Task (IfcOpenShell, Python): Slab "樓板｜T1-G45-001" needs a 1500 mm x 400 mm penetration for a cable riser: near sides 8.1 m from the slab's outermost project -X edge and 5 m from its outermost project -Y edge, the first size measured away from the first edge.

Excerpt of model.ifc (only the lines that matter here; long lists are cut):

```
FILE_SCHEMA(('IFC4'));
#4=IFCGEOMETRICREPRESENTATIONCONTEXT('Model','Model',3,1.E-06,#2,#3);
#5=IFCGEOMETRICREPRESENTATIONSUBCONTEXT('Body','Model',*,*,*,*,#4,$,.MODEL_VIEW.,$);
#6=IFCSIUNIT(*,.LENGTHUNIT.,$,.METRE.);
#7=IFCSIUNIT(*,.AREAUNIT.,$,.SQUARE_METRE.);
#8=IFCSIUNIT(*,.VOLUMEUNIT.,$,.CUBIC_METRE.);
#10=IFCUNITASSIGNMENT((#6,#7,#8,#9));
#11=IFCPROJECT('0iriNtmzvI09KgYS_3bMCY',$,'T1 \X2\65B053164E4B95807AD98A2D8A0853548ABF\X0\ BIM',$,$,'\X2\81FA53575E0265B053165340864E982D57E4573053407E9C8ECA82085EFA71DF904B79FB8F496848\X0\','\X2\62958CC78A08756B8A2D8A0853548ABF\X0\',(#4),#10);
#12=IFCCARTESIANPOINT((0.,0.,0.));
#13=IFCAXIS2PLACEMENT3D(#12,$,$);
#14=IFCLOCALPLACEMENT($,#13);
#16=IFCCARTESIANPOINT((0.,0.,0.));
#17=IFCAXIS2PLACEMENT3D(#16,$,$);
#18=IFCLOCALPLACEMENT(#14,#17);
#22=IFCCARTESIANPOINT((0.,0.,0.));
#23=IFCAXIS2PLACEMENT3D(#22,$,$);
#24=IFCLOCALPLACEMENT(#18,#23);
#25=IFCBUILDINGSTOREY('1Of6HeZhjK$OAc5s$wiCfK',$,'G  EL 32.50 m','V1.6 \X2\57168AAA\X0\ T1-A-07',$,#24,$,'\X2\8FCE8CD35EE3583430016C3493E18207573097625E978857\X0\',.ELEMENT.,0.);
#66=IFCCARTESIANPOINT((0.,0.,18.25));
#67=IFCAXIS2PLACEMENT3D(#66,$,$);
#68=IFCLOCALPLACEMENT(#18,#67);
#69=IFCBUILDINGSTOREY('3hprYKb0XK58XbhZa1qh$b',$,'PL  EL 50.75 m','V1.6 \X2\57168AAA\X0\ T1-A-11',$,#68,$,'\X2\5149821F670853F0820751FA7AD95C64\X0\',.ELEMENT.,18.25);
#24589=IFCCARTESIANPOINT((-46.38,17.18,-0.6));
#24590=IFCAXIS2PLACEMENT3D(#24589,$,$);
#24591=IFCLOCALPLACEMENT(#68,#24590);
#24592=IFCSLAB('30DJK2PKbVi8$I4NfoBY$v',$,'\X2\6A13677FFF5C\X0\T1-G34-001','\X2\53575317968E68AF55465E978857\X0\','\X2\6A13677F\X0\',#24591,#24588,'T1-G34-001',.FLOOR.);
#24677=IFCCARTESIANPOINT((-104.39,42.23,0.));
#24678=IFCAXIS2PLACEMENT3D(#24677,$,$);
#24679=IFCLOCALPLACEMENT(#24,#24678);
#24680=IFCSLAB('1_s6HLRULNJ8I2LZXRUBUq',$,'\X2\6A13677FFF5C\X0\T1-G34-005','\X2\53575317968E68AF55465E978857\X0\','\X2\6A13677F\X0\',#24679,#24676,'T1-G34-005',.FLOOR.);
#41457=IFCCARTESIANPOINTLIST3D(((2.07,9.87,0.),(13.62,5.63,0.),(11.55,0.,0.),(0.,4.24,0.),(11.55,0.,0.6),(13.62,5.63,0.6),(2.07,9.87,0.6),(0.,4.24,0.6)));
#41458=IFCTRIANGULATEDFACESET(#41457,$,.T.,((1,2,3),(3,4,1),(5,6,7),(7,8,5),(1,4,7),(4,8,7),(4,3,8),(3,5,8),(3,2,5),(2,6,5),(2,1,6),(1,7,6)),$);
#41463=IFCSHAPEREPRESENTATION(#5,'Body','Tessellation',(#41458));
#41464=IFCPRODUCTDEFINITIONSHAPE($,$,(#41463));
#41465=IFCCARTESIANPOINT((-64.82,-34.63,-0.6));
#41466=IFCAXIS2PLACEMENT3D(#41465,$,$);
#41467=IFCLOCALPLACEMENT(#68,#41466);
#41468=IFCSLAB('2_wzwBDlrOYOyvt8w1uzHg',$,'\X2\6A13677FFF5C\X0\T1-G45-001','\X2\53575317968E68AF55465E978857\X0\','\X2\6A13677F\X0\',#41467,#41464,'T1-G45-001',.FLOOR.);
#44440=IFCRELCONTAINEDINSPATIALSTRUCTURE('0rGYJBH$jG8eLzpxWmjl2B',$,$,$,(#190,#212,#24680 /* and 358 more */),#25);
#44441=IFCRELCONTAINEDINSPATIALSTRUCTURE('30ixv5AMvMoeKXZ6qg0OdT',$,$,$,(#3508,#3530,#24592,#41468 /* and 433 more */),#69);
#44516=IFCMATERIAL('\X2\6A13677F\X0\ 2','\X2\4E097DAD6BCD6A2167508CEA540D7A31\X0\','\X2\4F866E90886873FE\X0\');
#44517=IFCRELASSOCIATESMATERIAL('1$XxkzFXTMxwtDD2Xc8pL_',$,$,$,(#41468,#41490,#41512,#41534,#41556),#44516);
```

```python
import numpy as np
import ifcopenshell
import ifcopenshell.api.feature
import ifcopenshell.api.geometry
import ifcopenshell.api.root
import ifcopenshell.geom
import ifcopenshell.util.placement
import ifcopenshell.util.representation
import ifcopenshell.util.shape
import ifcopenshell.util.unit

model = ifcopenshell.open("model.ifc")
unit_scale = ifcopenshell.util.unit.calculate_unit_scale(model)
settings = ifcopenshell.geom.settings()


def volume(element):
    """Net volume in cubic metres, openings subtracted."""
    shape = ifcopenshell.geom.create_shape(settings, element)
    return ifcopenshell.util.shape.get_volume(shape.geometry)


slab = model.by_guid("2_wzwBDlrOYOyvt8w1uzHg")
before = volume(slab)

# Extent in the slab's own axes, in metres. The edges named are its -X and -Y sides.
slab_shape = ifcopenshell.geom.create_shape(settings, slab)
vertices = ifcopenshell.util.shape.get_vertices(slab_shape.geometry)
x_min, y_min, bottom = vertices.min(axis=0)
top = vertices[:, 2].max()

opening = ifcopenshell.api.root.create_entity(model, ifc_class="IfcOpeningElement", name="Cable riser opening", predefined_type="OPENING")
context = ifcopenshell.util.representation.get_context(model, "Model", "Body", "MODEL_VIEW")
width, depth = 1.5, 0.4
outline = [(0.0, 0.0), (width, 0.0), (width, depth), (0.0, depth), (0.0, 0.0)]
# Overshoot both faces by 50 mm so the cut is clean.
shape = ifcopenshell.api.geometry.add_slab_representation(
    model, context=context, depth=top - bottom + 0.1, polyline=outline
)
ifcopenshell.api.geometry.assign_representation(model, product=opening, representation=shape)

matrix = ifcopenshell.util.placement.get_local_placement(slab.ObjectPlacement)
matrix[:, 3] = matrix @ np.append(np.array([x_min + 8.1, y_min + 5, bottom - 0.05]) / unit_scale, 1.0)
ifcopenshell.api.geometry.edit_object_placement(model, product=opening, matrix=matrix, is_si=False)
ifcopenshell.api.feature.add_feature(model, feature=opening, element=slab)

after = volume(slab)

print(f"slab volume {before:.3f} -> {after:.3f} m3")

model.write("model_rev.ifc")
```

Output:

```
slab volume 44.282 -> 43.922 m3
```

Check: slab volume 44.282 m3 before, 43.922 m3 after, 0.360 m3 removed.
